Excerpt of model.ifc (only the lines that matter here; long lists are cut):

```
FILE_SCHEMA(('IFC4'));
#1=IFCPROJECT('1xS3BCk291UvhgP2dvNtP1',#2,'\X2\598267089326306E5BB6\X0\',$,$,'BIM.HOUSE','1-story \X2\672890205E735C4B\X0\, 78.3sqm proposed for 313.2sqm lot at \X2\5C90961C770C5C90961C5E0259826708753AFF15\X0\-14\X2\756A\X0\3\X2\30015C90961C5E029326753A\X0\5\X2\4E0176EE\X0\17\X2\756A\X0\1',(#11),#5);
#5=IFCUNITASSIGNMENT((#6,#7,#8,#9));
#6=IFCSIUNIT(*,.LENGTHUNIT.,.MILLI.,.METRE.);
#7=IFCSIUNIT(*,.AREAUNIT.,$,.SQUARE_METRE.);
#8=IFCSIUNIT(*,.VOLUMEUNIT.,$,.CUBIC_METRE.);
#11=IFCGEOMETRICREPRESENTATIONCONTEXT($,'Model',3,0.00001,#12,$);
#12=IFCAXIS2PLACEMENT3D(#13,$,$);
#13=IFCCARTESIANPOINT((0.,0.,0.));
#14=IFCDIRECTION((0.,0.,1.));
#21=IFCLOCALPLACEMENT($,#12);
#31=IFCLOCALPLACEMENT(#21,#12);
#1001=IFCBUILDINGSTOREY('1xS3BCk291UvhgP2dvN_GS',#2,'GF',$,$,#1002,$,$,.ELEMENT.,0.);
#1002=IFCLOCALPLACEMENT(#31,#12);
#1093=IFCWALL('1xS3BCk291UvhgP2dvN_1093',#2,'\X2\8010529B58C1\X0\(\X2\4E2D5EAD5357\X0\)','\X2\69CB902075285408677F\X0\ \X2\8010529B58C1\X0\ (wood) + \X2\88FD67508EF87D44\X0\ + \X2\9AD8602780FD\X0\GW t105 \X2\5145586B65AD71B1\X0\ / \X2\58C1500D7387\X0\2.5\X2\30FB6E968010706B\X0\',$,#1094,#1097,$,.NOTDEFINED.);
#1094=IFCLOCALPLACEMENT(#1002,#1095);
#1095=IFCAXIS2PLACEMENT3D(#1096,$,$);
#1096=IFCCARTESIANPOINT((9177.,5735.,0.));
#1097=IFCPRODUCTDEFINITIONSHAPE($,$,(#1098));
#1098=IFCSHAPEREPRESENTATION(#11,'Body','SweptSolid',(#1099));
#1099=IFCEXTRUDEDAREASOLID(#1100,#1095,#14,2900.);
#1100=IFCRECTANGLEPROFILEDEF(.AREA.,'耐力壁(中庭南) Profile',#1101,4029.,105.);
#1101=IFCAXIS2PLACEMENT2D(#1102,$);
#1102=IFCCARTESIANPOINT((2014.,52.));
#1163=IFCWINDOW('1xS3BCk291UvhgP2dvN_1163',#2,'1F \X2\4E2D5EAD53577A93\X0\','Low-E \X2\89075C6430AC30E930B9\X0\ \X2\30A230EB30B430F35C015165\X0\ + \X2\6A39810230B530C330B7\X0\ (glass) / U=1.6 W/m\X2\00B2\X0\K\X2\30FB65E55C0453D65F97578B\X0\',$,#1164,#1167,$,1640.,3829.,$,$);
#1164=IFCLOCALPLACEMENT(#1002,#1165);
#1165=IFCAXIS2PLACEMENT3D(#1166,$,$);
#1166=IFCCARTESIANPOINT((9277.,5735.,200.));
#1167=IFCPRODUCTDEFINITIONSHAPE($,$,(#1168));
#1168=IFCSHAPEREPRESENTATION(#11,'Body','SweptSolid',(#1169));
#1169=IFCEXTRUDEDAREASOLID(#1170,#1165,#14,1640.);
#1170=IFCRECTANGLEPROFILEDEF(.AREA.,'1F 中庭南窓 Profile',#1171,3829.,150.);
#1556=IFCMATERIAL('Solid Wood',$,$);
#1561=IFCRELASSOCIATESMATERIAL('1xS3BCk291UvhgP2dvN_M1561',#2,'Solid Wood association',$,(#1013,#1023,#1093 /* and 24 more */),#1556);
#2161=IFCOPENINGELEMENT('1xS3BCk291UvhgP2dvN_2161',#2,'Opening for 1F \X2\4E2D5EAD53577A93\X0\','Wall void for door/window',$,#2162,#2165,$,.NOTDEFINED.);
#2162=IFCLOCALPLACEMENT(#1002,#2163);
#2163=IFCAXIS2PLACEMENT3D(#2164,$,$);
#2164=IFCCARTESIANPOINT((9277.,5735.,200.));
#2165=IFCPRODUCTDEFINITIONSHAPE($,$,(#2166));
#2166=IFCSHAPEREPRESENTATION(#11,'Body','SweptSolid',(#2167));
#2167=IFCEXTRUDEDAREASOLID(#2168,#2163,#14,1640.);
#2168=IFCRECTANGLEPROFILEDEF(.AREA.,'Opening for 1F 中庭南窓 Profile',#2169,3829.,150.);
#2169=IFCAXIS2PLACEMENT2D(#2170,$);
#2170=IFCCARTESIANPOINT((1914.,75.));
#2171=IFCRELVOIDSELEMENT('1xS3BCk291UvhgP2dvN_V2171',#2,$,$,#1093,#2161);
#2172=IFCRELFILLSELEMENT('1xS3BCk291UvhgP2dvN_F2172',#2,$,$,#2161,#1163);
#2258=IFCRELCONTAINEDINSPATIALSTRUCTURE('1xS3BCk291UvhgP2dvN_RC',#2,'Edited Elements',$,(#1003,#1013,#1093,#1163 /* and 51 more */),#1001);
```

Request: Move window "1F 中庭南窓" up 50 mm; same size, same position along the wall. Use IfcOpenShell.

```python
import numpy as np
import ifcopenshell
import ifcopenshell.api.geometry
import ifcopenshell.util.placement
import ifcopenshell.util.unit

model = ifcopenshell.open("model.ifc")
unit_scale = ifcopenshell.util.unit.calculate_unit_scale(model)

window = model.by_guid("1xS3BCk291UvhgP2dvN_1163")
opening = window.FillsVoids[0].RelatingOpeningElement
dz = 0.05 / unit_scale

shift = np.array([0.0, 0.0, dz])
# The window is not placed relative to its opening, so move both.
for product in (opening, window):
    matrix = ifcopenshell.util.placement.get_local_placement(product.ObjectPlacement)
    matrix[:3, 3] += shift
    ifcopenshell.api.geometry.edit_object_placement(model, product=product, matrix=matrix, is_si=False)

print(f"moved by {dz * unit_scale:+.3f} m")

model.write("model_rev.ifc")
```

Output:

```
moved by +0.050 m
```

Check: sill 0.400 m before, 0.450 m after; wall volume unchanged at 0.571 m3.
